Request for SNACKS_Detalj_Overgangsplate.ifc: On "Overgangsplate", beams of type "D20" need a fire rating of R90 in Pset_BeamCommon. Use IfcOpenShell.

First a look at what the model holds.

```python
import ifcopenshell
import ifcopenshell.util.element

model = ifcopenshell.open("SNACKS_Detalj_Overgangsplate.ifc")
print(model.schema)
storey = next(s for s in model.by_type("IfcBuildingStorey") if s.Name == "Overgangsplate")
beams = [e for e in ifcopenshell.util.element.get_decomposition(storey) if e.is_a("IfcBeam")]
seen = {}
for e in beams:
    element_type = ifcopenshell.util.element.get_type(e)
    key = (element_type.Name if element_type != e and element_type else None, ifcopenshell.util.element.get_pset(e, "Pset_BeamCommon", "FireRating"))
    seen[key] = seen.get(key, 0) + 1
for (name, value), count in sorted(seen.items(), key=str):
    print(count, "x", name, "|", value)
```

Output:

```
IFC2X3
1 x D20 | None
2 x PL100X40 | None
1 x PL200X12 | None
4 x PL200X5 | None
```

```python
import ifcopenshell
import ifcopenshell.api.pset
import ifcopenshell.util.element

model = ifcopenshell.open("SNACKS_Detalj_Overgangsplate.ifc")

storey = next(s for s in model.by_type("IfcBuildingStorey") if s.Name == "Overgangsplate")
beams = [e for e in ifcopenshell.util.element.get_decomposition(storey) if e.is_a("IfcBeam")]

count = 0
for e in beams:
    element_type = ifcopenshell.util.element.get_type(e)
    if element_type in (None, e) or element_type.Name != "D20":
        continue
    # add_pset returns the element's existing set when there is one.
    pset = ifcopenshell.api.pset.add_pset(model, product=e, name="Pset_BeamCommon")
    ifcopenshell.api.pset.edit_pset(model, pset=pset, properties={"FireRating": "R90"})
    count += 1

print(count, "beams updated")

model.write("SNACKS_Detalj_Overgangsplate_edited.ifc")
```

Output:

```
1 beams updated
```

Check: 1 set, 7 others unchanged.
